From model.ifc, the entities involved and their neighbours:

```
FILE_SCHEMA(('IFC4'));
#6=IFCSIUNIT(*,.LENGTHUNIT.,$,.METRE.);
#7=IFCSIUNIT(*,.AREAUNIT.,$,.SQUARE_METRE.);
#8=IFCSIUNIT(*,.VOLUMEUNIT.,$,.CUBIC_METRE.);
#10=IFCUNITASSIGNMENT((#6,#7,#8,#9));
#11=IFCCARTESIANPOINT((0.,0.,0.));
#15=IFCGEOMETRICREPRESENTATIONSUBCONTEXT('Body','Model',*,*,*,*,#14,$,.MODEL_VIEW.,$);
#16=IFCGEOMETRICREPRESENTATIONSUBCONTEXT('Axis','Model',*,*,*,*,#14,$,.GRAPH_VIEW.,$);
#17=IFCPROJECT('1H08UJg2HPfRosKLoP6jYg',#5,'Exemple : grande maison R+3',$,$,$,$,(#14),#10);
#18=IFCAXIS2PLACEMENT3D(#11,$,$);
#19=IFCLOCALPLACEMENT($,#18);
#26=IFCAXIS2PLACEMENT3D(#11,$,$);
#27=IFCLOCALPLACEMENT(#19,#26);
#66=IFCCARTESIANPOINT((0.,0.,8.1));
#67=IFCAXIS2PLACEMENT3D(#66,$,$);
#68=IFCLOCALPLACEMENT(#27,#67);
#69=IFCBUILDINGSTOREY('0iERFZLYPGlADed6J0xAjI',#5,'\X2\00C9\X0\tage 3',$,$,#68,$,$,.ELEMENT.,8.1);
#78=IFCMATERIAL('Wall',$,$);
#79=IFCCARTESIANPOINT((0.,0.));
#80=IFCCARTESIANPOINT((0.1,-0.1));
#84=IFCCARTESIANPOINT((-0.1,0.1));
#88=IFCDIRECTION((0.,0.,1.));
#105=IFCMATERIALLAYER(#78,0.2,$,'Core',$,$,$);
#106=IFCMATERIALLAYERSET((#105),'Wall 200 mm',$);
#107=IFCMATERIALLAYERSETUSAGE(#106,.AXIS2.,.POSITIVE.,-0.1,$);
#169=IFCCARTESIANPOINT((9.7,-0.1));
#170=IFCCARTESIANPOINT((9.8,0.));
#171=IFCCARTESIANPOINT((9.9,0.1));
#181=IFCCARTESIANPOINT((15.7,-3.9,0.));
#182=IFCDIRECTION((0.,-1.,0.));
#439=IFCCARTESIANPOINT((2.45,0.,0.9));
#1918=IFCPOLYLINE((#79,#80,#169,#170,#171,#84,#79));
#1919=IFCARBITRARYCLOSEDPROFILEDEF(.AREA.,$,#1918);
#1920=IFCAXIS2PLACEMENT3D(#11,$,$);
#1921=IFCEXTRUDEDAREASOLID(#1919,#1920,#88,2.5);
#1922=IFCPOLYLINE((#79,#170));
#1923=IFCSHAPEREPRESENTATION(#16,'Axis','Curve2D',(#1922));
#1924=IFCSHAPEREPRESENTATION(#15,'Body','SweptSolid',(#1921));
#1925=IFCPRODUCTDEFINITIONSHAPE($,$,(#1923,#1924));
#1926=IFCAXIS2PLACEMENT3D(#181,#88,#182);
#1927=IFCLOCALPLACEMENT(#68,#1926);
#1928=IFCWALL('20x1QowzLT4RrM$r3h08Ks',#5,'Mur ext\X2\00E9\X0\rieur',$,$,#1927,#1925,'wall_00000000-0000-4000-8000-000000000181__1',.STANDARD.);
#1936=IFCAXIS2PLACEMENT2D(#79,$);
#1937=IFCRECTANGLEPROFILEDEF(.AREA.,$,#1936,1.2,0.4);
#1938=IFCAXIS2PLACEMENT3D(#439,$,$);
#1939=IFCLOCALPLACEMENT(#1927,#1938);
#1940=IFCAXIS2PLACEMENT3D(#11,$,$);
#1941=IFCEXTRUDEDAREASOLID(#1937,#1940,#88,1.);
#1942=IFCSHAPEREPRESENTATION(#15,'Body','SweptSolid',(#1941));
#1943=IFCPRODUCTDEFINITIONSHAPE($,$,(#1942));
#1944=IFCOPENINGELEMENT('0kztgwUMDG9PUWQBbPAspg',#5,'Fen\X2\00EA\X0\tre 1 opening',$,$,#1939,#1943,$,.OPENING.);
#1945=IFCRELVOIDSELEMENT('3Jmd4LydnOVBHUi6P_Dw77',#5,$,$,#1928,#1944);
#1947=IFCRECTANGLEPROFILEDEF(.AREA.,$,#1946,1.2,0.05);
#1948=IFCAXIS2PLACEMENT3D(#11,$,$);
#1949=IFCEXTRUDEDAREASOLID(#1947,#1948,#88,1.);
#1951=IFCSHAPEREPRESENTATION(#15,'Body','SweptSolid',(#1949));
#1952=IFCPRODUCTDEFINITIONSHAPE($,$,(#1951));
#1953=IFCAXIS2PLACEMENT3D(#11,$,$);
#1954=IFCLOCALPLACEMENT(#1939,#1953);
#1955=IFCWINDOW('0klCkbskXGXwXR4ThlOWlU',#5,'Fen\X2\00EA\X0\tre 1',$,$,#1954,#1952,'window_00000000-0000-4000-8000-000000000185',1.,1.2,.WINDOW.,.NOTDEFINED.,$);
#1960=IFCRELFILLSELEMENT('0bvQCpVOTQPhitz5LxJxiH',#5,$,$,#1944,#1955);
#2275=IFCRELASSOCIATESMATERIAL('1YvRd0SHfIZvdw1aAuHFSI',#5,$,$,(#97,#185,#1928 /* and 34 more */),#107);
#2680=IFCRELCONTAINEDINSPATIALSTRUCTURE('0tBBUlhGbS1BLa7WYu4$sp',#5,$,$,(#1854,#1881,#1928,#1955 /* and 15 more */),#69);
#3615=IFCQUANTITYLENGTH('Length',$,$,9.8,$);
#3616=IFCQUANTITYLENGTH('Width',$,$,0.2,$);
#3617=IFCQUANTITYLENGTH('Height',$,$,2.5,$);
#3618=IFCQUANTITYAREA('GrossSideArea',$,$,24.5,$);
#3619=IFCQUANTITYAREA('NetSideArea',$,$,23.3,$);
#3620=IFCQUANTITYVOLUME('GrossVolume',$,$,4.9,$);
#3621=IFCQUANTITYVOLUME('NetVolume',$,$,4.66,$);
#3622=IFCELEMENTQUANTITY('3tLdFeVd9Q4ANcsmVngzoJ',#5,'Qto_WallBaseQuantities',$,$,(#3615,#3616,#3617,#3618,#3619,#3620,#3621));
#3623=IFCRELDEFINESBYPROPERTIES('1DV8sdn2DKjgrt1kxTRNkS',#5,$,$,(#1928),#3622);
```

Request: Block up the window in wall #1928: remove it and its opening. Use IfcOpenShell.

```python
import ifcopenshell
import ifcopenshell.api.feature
import ifcopenshell.api.pset
import ifcopenshell.api.root
import ifcopenshell.geom
import ifcopenshell.util.element
import ifcopenshell.util.shape
import ifcopenshell.util.unit

model = ifcopenshell.open("model.ifc")
area_scale = ifcopenshell.util.unit.calculate_unit_scale(model, "AREAUNIT")
volume_scale = ifcopenshell.util.unit.calculate_unit_scale(model, "VOLUMEUNIT")
settings = ifcopenshell.geom.settings()


def volume(element):
    """Net volume in cubic metres, openings subtracted."""
    shape = ifcopenshell.geom.create_shape(settings, element)
    return ifcopenshell.util.shape.get_volume(shape.geometry)


window = model.by_guid("0klCkbskXGXwXR4ThlOWlU")
opening = window.FillsVoids[0].RelatingOpeningElement
wall = opening.VoidsElements[0].RelatingBuildingElement
before = volume(wall)

ifcopenshell.api.root.remove_product(model, product=window)
ifcopenshell.api.feature.remove_feature(model, feature=opening)

after = volume(wall)
thickness = 0.2  # wall thickness in metres

# Update the wall's stored quantities.
qto = model.by_id(ifcopenshell.util.element.get_pset(wall, "Qto_WallBaseQuantities", should_inherit=False)["id"])
ifcopenshell.api.pset.edit_qto(model, qto=qto, properties={
    "NetSideArea": after / thickness / area_scale,
    "NetVolume": after / volume_scale,
})

print(f"wall volume {before:.3f} -> {after:.3f} m3")

model.write("model_rev.ifc")
```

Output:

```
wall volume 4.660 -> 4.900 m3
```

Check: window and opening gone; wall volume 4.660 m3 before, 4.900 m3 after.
